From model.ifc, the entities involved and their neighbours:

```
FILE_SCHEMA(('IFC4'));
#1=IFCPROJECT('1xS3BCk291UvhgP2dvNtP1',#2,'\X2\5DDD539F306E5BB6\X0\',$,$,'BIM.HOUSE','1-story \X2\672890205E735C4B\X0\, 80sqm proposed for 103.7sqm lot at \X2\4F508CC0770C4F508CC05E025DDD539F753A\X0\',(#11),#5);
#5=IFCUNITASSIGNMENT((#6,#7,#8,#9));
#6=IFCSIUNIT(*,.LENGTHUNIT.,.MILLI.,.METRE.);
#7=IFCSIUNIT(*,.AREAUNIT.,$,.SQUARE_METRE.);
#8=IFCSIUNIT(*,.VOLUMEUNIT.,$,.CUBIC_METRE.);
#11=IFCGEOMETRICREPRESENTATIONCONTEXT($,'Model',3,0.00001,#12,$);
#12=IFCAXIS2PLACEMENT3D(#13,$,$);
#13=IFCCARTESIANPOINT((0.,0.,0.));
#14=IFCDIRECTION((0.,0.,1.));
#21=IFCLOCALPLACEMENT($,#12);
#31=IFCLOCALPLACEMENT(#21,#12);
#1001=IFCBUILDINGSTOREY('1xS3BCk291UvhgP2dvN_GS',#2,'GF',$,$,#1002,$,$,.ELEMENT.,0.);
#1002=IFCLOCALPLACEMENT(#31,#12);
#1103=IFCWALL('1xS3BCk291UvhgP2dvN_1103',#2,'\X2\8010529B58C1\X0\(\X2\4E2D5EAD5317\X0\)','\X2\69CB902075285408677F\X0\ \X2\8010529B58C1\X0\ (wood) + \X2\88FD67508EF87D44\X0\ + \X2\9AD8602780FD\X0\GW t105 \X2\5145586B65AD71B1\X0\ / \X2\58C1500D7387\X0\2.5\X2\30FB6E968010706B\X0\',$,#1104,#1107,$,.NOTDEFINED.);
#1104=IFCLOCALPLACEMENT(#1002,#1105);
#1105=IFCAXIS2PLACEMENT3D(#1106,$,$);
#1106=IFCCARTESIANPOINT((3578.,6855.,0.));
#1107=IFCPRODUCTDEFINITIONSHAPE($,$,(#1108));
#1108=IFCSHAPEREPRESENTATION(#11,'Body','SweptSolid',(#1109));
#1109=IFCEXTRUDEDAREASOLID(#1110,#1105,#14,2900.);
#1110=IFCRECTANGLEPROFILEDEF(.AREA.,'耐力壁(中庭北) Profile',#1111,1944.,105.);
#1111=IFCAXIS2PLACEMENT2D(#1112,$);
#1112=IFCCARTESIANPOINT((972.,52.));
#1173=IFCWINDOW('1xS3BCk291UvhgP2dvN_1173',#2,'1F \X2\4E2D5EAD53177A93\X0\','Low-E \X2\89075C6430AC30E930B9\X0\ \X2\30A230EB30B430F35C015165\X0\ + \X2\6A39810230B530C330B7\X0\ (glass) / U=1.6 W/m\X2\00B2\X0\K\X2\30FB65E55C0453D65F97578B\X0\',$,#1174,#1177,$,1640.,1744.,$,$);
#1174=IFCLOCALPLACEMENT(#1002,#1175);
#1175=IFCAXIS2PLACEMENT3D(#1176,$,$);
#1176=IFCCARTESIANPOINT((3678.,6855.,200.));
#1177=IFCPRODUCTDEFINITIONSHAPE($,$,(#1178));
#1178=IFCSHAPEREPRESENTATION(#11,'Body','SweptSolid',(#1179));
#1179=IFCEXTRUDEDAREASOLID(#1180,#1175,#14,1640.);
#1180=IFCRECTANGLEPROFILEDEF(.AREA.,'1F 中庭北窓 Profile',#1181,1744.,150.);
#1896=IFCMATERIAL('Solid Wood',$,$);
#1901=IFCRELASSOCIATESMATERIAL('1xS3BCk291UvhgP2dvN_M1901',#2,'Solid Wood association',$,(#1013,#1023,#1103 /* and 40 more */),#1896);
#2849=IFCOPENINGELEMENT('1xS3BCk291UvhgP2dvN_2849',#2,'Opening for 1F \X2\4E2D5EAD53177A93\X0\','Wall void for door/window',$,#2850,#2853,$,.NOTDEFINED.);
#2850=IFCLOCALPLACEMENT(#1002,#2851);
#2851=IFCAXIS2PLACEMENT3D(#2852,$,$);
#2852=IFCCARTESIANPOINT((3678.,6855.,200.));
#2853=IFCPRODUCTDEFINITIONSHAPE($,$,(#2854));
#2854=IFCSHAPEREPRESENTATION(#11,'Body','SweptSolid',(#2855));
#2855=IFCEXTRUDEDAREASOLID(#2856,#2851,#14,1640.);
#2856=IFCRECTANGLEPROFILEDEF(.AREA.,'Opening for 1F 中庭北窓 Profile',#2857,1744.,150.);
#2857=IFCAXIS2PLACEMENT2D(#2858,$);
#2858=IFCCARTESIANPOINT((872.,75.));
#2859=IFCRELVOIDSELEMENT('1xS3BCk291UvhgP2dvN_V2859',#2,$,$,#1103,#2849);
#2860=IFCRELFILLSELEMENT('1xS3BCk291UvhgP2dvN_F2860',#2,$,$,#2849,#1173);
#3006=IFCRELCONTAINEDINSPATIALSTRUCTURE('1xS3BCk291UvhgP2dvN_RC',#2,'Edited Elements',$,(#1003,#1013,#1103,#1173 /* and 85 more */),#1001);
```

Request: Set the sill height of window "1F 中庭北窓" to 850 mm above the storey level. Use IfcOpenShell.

```python
import numpy as np
import ifcopenshell
import ifcopenshell.api.geometry
import ifcopenshell.geom
import ifcopenshell.util.element
import ifcopenshell.util.placement
import ifcopenshell.util.shape
import ifcopenshell.util.unit

model = ifcopenshell.open("model.ifc")
unit_scale = ifcopenshell.util.unit.calculate_unit_scale(model)

window = model.by_guid("1xS3BCk291UvhgP2dvN_1173")
opening = window.FillsVoids[0].RelatingOpeningElement
storey = ifcopenshell.util.element.get_container(window, ifc_class="IfcBuildingStorey")
level = ifcopenshell.util.placement.get_local_placement(storey.ObjectPlacement)[2, 3]

# The opening's origin need not be at the sill, so measure its lowest point.
shape = ifcopenshell.geom.create_shape(ifcopenshell.geom.settings(), opening)
bottom = ifcopenshell.util.shape.get_shape_bottom_elevation(shape, shape.geometry) / unit_scale
dz = level + 850.0 - bottom

shift = np.array([0.0, 0.0, dz])
# The window is not placed relative to its opening, so move both.
for product in (opening, window):
    matrix = ifcopenshell.util.placement.get_local_placement(product.ObjectPlacement)
    matrix[:3, 3] += shift
    ifcopenshell.api.geometry.edit_object_placement(model, product=product, matrix=matrix, is_si=False)

print(f"moved by {dz * unit_scale:+.3f} m")

model.write("model_rev.ifc")
```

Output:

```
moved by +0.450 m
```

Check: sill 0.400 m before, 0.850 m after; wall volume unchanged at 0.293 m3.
